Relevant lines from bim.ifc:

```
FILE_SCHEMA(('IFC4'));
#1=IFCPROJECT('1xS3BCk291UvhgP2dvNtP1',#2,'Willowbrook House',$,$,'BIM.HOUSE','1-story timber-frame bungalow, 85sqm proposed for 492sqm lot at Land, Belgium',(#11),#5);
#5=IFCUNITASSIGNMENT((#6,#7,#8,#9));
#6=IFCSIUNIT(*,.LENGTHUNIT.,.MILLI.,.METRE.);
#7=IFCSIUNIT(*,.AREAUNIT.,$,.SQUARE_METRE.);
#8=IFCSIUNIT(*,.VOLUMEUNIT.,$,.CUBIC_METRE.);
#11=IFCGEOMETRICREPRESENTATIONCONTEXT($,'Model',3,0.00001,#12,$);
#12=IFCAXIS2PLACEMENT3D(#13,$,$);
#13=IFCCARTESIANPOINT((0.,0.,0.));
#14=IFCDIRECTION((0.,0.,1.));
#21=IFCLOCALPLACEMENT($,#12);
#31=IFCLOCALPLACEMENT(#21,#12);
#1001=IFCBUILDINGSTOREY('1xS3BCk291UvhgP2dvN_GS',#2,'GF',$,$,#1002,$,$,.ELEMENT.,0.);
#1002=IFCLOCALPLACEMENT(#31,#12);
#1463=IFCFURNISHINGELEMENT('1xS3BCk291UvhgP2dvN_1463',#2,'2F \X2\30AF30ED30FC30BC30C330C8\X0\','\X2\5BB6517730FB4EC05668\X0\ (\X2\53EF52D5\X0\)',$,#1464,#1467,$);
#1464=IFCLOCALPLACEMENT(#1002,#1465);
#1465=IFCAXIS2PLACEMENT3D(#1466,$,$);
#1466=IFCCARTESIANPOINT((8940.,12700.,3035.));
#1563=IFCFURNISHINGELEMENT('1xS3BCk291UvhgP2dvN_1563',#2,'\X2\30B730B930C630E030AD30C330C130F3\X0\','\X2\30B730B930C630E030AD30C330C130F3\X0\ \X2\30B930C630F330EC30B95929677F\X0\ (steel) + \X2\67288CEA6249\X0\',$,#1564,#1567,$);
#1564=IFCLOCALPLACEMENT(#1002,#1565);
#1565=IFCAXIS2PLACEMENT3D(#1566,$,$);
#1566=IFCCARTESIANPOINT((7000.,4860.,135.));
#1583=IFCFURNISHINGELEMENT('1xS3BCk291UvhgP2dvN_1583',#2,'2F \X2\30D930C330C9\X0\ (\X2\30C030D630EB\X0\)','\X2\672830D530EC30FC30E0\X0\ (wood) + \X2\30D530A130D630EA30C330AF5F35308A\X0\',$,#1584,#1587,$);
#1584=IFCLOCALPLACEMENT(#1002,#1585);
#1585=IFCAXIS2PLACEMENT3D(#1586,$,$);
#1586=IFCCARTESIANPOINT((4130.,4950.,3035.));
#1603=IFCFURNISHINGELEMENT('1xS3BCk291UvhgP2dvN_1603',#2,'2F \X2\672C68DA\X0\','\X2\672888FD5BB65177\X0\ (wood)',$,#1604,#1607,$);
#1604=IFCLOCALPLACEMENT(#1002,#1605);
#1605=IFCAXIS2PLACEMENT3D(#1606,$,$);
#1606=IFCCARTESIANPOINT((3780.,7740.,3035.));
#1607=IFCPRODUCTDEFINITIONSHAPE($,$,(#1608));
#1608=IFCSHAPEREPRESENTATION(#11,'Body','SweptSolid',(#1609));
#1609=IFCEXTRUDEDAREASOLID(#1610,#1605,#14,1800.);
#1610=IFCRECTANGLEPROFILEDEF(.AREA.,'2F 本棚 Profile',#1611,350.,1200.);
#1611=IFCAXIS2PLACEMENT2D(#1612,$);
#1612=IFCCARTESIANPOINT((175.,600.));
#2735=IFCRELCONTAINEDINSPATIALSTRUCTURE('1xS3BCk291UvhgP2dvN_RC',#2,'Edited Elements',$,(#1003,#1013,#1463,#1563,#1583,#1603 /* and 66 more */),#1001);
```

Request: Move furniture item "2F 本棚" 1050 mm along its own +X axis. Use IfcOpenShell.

```python
import ifcopenshell
import ifcopenshell.api.geometry
import ifcopenshell.util.placement
import ifcopenshell.util.unit

model = ifcopenshell.open("bim.ifc")
unit_scale = ifcopenshell.util.unit.calculate_unit_scale(model)

item = model.by_id(1603)
matrix = ifcopenshell.util.placement.get_local_placement(item.ObjectPlacement)
matrix[:3, 3] += matrix[:3, 0] * 1.05 / unit_scale
ifcopenshell.api.geometry.edit_object_placement(model, product=item, matrix=matrix, is_si=False)

print(ifcopenshell.util.placement.get_local_placement(item.ObjectPlacement).round(3) + 0.0)

model.write("bim_rev.ifc")
```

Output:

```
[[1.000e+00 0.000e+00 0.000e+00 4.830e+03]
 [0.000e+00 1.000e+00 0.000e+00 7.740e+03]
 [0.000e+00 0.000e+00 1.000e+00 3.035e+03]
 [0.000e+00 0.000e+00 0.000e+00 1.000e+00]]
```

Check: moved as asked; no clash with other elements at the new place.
